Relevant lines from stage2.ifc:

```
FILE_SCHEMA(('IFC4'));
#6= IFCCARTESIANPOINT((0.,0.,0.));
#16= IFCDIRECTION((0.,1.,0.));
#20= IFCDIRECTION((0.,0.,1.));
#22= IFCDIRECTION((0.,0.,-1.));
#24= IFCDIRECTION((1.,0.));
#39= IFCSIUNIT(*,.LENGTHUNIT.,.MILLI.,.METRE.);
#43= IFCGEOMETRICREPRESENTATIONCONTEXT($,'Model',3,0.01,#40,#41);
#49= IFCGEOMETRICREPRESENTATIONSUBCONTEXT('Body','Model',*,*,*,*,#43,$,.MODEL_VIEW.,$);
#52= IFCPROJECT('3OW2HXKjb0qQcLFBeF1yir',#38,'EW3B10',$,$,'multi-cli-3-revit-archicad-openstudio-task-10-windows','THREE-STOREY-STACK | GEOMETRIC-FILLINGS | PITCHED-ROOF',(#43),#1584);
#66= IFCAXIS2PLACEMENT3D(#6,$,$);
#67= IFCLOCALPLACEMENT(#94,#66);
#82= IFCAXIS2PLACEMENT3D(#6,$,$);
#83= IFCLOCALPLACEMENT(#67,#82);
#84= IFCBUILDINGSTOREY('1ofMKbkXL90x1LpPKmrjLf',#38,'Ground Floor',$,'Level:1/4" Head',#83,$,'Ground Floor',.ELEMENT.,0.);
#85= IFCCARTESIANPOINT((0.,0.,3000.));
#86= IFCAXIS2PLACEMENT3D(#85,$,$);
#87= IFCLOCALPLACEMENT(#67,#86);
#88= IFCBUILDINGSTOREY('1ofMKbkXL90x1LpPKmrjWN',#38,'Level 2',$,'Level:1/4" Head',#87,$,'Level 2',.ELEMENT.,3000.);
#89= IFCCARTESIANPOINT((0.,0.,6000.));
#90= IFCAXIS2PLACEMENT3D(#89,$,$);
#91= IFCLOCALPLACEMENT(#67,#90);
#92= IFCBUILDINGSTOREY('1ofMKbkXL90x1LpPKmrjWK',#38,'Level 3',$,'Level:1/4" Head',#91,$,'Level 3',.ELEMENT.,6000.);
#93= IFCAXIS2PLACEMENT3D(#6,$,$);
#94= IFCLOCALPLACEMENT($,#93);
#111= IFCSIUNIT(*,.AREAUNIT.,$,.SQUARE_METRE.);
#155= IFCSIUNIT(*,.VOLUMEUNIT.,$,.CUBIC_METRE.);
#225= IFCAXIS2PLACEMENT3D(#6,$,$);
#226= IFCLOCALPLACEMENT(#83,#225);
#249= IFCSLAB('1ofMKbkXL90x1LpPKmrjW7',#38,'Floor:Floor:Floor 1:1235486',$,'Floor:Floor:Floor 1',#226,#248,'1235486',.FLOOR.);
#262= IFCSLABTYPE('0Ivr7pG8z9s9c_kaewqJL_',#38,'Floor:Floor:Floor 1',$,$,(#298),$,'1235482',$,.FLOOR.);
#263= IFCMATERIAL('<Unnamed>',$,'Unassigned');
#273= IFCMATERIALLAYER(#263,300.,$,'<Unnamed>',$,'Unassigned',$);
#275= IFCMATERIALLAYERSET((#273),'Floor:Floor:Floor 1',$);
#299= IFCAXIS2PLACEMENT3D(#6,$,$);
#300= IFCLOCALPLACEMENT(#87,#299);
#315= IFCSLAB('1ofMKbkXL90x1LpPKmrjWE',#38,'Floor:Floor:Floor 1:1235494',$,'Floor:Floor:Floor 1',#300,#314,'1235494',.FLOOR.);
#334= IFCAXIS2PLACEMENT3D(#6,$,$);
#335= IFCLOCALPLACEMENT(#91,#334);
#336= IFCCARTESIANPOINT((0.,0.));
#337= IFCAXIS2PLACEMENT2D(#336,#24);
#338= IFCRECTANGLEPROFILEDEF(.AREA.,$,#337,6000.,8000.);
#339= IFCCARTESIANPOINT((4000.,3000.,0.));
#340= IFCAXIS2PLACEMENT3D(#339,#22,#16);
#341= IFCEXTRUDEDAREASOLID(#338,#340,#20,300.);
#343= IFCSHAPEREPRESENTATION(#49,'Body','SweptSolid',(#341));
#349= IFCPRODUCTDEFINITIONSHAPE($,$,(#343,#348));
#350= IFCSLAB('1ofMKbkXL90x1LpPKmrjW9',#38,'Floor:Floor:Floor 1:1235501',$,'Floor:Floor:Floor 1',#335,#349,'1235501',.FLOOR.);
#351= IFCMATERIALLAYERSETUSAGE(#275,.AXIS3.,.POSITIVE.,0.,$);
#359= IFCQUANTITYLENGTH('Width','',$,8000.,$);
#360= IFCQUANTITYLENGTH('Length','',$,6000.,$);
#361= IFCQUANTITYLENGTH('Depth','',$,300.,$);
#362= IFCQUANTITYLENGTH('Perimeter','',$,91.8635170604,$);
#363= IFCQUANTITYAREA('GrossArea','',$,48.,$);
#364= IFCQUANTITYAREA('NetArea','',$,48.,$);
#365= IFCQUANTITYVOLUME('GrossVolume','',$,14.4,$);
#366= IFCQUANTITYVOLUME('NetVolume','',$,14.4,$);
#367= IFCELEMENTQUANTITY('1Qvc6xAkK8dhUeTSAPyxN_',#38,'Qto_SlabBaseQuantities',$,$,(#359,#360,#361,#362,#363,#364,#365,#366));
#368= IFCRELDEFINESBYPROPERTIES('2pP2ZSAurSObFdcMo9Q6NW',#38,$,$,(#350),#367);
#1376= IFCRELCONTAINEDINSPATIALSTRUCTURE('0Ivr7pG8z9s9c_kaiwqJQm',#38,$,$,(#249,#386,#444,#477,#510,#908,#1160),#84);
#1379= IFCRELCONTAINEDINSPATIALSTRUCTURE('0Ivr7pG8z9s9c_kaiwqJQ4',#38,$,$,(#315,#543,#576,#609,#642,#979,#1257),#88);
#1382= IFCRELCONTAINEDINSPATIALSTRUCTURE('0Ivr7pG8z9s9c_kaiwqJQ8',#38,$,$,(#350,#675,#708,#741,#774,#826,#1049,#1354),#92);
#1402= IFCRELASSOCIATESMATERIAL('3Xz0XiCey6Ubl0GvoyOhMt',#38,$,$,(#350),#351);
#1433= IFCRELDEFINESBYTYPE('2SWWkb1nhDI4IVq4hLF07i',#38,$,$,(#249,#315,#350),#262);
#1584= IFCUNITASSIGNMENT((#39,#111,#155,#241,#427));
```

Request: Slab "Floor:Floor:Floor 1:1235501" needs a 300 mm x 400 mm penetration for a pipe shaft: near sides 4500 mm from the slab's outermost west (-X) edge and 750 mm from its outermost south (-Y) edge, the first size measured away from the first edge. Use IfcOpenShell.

```python
import numpy as np
import ifcopenshell
import ifcopenshell.api.feature
import ifcopenshell.api.geometry
import ifcopenshell.api.pset
import ifcopenshell.api.root
import ifcopenshell.geom
import ifcopenshell.util.element
import ifcopenshell.util.placement
import ifcopenshell.util.representation
import ifcopenshell.util.shape
import ifcopenshell.util.unit

model = ifcopenshell.open("stage2.ifc")
unit_scale = ifcopenshell.util.unit.calculate_unit_scale(model)
area_scale = ifcopenshell.util.unit.calculate_unit_scale(model, "AREAUNIT")
volume_scale = ifcopenshell.util.unit.calculate_unit_scale(model, "VOLUMEUNIT")
settings = ifcopenshell.geom.settings()


def volume(element):
    """Net volume in cubic metres, openings subtracted."""
    shape = ifcopenshell.geom.create_shape(settings, element)
    return ifcopenshell.util.shape.get_volume(shape.geometry)


slab = model.by_id(350)
before = volume(slab)

# Extent in the slab's own axes, in metres. The edges named are its -X and -Y sides.
slab_shape = ifcopenshell.geom.create_shape(settings, slab)
vertices = ifcopenshell.util.shape.get_vertices(slab_shape.geometry)
x_min, y_min, bottom = vertices.min(axis=0)
top = vertices[:, 2].max()

opening = ifcopenshell.api.root.create_entity(model, ifc_class="IfcOpeningElement", name="Pipe shaft opening", predefined_type="OPENING")
context = ifcopenshell.util.representation.get_context(model, "Model", "Body", "MODEL_VIEW")
width, depth = 0.3, 0.4
outline = [(0.0, 0.0), (width, 0.0), (width, depth), (0.0, depth), (0.0, 0.0)]
# Overshoot both faces by 50 mm so the cut is clean.
shape = ifcopenshell.api.geometry.add_slab_representation(
    model, context=context, depth=top - bottom + 0.1, polyline=outline
)
ifcopenshell.api.geometry.assign_representation(model, product=opening, representation=shape)

matrix = ifcopenshell.util.placement.get_local_placement(slab.ObjectPlacement)
matrix[:, 3] = matrix @ np.append(np.array([x_min + 4.5, y_min + 0.75, bottom - 0.05]) / unit_scale, 1.0)
ifcopenshell.api.geometry.edit_object_placement(model, product=opening, matrix=matrix, is_si=False)
ifcopenshell.api.feature.add_feature(model, feature=opening, element=slab)

after = volume(slab)

# Update the slab's stored quantities.
qto = model.by_id(ifcopenshell.util.element.get_pset(slab, "Qto_SlabBaseQuantities", should_inherit=False)["id"])
ifcopenshell.api.pset.edit_qto(model, qto=qto, properties={
    "NetArea": after / (top - bottom) / area_scale,
    "NetVolume": after / volume_scale,
})

print(f"slab volume {before:.3f} -> {after:.3f} m3")

model.write("stage2_rev.ifc")
```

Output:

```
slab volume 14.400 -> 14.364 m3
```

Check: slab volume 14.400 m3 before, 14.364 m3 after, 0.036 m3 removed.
